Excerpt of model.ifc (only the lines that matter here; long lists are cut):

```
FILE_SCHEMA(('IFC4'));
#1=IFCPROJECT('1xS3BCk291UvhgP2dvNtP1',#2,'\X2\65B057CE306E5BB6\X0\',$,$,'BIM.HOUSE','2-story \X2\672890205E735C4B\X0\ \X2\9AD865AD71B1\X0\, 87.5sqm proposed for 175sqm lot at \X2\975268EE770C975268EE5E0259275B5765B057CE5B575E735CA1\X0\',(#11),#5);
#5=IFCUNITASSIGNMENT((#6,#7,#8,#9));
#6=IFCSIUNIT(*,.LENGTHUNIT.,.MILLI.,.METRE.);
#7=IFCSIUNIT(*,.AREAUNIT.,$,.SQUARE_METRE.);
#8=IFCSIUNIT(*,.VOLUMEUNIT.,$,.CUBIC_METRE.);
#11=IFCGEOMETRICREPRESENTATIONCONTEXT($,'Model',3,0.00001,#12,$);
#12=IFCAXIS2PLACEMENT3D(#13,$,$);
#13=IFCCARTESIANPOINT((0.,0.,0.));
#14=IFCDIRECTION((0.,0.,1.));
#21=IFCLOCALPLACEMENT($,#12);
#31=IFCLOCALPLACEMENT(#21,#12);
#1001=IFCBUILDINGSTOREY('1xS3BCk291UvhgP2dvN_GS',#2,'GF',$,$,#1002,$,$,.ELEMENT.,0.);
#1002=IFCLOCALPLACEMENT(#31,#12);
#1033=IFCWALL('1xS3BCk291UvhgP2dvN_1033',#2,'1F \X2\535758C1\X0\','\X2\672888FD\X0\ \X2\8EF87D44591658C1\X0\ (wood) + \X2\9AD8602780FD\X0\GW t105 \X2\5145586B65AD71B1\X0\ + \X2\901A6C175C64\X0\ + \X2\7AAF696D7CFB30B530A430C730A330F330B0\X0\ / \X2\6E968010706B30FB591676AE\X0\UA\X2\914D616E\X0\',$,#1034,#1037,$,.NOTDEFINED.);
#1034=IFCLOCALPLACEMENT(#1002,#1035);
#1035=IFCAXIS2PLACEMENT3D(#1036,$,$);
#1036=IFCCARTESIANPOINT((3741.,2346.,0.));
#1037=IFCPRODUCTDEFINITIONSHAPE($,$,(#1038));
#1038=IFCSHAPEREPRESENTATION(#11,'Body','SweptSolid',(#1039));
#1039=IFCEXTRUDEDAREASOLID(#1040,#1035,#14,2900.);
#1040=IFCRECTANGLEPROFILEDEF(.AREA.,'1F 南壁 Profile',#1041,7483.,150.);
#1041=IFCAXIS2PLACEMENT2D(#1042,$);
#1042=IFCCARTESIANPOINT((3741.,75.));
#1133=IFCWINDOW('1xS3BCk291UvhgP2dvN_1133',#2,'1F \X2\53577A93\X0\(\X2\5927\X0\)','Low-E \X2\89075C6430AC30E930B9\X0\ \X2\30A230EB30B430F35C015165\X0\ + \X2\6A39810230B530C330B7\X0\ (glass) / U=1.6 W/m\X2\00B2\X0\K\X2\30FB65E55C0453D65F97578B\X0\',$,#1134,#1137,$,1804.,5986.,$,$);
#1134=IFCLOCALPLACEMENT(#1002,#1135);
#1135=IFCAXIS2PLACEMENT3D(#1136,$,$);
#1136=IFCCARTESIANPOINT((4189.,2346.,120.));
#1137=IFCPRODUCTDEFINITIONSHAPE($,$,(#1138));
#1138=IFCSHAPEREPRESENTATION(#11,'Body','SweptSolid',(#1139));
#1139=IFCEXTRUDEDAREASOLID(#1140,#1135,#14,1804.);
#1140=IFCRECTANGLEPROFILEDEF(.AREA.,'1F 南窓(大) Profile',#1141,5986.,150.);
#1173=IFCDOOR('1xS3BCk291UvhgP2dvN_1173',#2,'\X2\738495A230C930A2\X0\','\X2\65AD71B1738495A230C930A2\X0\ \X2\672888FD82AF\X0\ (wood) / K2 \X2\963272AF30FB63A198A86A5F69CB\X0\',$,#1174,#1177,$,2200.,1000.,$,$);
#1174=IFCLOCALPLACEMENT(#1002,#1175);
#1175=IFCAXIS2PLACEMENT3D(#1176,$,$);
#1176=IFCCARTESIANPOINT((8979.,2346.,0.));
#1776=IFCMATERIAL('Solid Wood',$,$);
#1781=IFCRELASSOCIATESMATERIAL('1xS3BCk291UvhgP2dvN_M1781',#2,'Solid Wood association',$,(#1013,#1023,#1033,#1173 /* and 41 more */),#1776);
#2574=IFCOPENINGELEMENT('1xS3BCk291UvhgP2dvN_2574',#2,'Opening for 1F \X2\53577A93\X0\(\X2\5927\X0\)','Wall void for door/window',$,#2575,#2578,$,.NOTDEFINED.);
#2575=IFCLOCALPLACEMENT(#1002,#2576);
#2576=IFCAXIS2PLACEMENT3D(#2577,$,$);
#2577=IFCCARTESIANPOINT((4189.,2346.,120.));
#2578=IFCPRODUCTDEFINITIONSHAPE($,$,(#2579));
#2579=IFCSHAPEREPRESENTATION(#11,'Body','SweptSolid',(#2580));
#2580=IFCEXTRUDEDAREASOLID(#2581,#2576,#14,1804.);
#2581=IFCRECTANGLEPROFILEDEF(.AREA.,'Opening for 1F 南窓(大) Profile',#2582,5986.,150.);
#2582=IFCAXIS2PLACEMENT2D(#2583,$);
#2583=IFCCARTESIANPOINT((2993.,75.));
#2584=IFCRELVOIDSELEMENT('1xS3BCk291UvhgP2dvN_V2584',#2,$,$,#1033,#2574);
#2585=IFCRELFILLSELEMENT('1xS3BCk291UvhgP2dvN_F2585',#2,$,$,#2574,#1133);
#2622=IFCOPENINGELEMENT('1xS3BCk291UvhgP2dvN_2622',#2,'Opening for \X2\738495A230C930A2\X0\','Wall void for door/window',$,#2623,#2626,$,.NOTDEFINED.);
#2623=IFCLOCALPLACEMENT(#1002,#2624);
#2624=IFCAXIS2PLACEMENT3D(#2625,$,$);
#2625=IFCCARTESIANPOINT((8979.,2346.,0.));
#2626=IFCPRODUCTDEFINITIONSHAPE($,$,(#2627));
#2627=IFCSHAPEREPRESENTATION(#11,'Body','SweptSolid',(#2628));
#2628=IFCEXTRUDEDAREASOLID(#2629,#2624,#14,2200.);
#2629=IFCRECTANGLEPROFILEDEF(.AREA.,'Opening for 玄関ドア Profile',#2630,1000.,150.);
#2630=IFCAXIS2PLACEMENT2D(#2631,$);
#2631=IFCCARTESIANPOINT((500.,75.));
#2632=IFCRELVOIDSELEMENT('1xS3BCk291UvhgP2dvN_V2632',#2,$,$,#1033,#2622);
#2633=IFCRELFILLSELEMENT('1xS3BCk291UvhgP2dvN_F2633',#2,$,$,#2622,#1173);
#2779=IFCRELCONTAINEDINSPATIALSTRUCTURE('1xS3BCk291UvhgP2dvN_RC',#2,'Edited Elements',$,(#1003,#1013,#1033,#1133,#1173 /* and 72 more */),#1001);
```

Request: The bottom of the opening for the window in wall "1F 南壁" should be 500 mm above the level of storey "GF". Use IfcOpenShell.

```python
import numpy as np
import ifcopenshell
import ifcopenshell.api.geometry
import ifcopenshell.geom
import ifcopenshell.util.element
import ifcopenshell.util.placement
import ifcopenshell.util.shape
import ifcopenshell.util.unit

model = ifcopenshell.open("model.ifc")
unit_scale = ifcopenshell.util.unit.calculate_unit_scale(model)

window = model.by_guid("1xS3BCk291UvhgP2dvN_1133")
opening = window.FillsVoids[0].RelatingOpeningElement
storey = ifcopenshell.util.element.get_container(window, ifc_class="IfcBuildingStorey")
level = ifcopenshell.util.placement.get_local_placement(storey.ObjectPlacement)[2, 3]

# The opening's origin need not be at the sill, so measure its lowest point.
shape = ifcopenshell.geom.create_shape(ifcopenshell.geom.settings(), opening)
bottom = ifcopenshell.util.shape.get_shape_bottom_elevation(shape, shape.geometry) / unit_scale
dz = level + 500.0 - bottom

shift = np.array([0.0, 0.0, dz])
# The window is not placed relative to its opening, so move both.
for product in (opening, window):
    matrix = ifcopenshell.util.placement.get_local_placement(product.ObjectPlacement)
    matrix[:3, 3] += shift
    ifcopenshell.api.geometry.edit_object_placement(model, product=product, matrix=matrix, is_si=False)

print(f"moved by {dz * unit_scale:+.3f} m")

model.write("model_rev.ifc")
```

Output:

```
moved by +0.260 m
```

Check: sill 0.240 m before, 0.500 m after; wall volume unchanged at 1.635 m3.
